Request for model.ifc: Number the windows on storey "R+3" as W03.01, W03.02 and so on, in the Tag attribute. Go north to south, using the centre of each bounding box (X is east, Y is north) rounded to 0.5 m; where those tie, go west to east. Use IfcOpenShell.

First a look at what the model holds.

```python
import ifcopenshell
import ifcopenshell.util.element
import ifcopenshell.util.placement

model = ifcopenshell.open("model.ifc")
print(model.schema)
storey = next(s for s in model.by_type("IfcBuildingStorey") if s.Name == "R+3")
windows = [e for e in ifcopenshell.util.element.get_decomposition(storey) if e.is_a("IfcWindow")]
for e in sorted(windows, key=lambda e: e.id()):
    origin = ifcopenshell.util.placement.get_local_placement(e.ObjectPlacement)[:3, 3]
    print(e.id(), e.Tag, e.Name, origin.round(2) + 0.0, sep=" | ")
```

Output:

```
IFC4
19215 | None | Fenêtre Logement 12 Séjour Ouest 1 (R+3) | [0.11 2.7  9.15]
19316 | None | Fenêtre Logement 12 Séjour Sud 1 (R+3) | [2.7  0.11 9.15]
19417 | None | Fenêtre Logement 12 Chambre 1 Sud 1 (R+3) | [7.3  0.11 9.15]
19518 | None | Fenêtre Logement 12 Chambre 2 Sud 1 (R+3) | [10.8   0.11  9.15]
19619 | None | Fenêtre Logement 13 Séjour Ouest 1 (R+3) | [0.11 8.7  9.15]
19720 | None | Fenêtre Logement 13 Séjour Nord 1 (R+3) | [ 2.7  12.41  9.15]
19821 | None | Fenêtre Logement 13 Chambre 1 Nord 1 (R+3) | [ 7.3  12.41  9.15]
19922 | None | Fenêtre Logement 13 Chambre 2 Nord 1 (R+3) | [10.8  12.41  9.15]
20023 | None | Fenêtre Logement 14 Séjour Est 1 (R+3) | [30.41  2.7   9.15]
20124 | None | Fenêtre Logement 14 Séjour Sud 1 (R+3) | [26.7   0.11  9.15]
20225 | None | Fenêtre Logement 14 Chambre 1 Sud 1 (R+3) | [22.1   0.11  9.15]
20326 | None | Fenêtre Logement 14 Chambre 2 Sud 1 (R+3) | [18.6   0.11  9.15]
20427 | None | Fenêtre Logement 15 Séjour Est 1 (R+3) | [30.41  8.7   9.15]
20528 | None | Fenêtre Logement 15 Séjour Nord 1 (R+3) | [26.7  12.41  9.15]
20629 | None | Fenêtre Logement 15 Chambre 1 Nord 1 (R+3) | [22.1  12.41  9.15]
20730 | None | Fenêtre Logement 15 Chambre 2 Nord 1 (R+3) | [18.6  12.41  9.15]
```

```python
import ifcopenshell
import ifcopenshell.geom
import ifcopenshell.util.element
import ifcopenshell.util.shape

model = ifcopenshell.open("model.ifc")
settings = ifcopenshell.geom.settings()
settings.set("use-world-coords", True)


def centre(element):
    shape = ifcopenshell.geom.create_shape(settings, element)
    return ifcopenshell.util.shape.get_bbox_centroid(shape.geometry)


storey = next(s for s in model.by_type("IfcBuildingStorey") if s.Name == "R+3")
windows = [e for e in ifcopenshell.util.element.get_decomposition(storey) if e.is_a("IfcWindow")]

# Insertion points can sit at a corner or the storey origin, so sort by the geometry (in metres).
centres = {e: centre(e) for e in windows}
windows.sort(key=lambda e: (-round(centres[e][1] / 0.5), centres[e][0]))

for i, e in enumerate(windows, start=1):
    number = f"W03.{i:02d}"
    e.Tag = number
    print(e.id(), number)

model.write("model_edited.ifc")
```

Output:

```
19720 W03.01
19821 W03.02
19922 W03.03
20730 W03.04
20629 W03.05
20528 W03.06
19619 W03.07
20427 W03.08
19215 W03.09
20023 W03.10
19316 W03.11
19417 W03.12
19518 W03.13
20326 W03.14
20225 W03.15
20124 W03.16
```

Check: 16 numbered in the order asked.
